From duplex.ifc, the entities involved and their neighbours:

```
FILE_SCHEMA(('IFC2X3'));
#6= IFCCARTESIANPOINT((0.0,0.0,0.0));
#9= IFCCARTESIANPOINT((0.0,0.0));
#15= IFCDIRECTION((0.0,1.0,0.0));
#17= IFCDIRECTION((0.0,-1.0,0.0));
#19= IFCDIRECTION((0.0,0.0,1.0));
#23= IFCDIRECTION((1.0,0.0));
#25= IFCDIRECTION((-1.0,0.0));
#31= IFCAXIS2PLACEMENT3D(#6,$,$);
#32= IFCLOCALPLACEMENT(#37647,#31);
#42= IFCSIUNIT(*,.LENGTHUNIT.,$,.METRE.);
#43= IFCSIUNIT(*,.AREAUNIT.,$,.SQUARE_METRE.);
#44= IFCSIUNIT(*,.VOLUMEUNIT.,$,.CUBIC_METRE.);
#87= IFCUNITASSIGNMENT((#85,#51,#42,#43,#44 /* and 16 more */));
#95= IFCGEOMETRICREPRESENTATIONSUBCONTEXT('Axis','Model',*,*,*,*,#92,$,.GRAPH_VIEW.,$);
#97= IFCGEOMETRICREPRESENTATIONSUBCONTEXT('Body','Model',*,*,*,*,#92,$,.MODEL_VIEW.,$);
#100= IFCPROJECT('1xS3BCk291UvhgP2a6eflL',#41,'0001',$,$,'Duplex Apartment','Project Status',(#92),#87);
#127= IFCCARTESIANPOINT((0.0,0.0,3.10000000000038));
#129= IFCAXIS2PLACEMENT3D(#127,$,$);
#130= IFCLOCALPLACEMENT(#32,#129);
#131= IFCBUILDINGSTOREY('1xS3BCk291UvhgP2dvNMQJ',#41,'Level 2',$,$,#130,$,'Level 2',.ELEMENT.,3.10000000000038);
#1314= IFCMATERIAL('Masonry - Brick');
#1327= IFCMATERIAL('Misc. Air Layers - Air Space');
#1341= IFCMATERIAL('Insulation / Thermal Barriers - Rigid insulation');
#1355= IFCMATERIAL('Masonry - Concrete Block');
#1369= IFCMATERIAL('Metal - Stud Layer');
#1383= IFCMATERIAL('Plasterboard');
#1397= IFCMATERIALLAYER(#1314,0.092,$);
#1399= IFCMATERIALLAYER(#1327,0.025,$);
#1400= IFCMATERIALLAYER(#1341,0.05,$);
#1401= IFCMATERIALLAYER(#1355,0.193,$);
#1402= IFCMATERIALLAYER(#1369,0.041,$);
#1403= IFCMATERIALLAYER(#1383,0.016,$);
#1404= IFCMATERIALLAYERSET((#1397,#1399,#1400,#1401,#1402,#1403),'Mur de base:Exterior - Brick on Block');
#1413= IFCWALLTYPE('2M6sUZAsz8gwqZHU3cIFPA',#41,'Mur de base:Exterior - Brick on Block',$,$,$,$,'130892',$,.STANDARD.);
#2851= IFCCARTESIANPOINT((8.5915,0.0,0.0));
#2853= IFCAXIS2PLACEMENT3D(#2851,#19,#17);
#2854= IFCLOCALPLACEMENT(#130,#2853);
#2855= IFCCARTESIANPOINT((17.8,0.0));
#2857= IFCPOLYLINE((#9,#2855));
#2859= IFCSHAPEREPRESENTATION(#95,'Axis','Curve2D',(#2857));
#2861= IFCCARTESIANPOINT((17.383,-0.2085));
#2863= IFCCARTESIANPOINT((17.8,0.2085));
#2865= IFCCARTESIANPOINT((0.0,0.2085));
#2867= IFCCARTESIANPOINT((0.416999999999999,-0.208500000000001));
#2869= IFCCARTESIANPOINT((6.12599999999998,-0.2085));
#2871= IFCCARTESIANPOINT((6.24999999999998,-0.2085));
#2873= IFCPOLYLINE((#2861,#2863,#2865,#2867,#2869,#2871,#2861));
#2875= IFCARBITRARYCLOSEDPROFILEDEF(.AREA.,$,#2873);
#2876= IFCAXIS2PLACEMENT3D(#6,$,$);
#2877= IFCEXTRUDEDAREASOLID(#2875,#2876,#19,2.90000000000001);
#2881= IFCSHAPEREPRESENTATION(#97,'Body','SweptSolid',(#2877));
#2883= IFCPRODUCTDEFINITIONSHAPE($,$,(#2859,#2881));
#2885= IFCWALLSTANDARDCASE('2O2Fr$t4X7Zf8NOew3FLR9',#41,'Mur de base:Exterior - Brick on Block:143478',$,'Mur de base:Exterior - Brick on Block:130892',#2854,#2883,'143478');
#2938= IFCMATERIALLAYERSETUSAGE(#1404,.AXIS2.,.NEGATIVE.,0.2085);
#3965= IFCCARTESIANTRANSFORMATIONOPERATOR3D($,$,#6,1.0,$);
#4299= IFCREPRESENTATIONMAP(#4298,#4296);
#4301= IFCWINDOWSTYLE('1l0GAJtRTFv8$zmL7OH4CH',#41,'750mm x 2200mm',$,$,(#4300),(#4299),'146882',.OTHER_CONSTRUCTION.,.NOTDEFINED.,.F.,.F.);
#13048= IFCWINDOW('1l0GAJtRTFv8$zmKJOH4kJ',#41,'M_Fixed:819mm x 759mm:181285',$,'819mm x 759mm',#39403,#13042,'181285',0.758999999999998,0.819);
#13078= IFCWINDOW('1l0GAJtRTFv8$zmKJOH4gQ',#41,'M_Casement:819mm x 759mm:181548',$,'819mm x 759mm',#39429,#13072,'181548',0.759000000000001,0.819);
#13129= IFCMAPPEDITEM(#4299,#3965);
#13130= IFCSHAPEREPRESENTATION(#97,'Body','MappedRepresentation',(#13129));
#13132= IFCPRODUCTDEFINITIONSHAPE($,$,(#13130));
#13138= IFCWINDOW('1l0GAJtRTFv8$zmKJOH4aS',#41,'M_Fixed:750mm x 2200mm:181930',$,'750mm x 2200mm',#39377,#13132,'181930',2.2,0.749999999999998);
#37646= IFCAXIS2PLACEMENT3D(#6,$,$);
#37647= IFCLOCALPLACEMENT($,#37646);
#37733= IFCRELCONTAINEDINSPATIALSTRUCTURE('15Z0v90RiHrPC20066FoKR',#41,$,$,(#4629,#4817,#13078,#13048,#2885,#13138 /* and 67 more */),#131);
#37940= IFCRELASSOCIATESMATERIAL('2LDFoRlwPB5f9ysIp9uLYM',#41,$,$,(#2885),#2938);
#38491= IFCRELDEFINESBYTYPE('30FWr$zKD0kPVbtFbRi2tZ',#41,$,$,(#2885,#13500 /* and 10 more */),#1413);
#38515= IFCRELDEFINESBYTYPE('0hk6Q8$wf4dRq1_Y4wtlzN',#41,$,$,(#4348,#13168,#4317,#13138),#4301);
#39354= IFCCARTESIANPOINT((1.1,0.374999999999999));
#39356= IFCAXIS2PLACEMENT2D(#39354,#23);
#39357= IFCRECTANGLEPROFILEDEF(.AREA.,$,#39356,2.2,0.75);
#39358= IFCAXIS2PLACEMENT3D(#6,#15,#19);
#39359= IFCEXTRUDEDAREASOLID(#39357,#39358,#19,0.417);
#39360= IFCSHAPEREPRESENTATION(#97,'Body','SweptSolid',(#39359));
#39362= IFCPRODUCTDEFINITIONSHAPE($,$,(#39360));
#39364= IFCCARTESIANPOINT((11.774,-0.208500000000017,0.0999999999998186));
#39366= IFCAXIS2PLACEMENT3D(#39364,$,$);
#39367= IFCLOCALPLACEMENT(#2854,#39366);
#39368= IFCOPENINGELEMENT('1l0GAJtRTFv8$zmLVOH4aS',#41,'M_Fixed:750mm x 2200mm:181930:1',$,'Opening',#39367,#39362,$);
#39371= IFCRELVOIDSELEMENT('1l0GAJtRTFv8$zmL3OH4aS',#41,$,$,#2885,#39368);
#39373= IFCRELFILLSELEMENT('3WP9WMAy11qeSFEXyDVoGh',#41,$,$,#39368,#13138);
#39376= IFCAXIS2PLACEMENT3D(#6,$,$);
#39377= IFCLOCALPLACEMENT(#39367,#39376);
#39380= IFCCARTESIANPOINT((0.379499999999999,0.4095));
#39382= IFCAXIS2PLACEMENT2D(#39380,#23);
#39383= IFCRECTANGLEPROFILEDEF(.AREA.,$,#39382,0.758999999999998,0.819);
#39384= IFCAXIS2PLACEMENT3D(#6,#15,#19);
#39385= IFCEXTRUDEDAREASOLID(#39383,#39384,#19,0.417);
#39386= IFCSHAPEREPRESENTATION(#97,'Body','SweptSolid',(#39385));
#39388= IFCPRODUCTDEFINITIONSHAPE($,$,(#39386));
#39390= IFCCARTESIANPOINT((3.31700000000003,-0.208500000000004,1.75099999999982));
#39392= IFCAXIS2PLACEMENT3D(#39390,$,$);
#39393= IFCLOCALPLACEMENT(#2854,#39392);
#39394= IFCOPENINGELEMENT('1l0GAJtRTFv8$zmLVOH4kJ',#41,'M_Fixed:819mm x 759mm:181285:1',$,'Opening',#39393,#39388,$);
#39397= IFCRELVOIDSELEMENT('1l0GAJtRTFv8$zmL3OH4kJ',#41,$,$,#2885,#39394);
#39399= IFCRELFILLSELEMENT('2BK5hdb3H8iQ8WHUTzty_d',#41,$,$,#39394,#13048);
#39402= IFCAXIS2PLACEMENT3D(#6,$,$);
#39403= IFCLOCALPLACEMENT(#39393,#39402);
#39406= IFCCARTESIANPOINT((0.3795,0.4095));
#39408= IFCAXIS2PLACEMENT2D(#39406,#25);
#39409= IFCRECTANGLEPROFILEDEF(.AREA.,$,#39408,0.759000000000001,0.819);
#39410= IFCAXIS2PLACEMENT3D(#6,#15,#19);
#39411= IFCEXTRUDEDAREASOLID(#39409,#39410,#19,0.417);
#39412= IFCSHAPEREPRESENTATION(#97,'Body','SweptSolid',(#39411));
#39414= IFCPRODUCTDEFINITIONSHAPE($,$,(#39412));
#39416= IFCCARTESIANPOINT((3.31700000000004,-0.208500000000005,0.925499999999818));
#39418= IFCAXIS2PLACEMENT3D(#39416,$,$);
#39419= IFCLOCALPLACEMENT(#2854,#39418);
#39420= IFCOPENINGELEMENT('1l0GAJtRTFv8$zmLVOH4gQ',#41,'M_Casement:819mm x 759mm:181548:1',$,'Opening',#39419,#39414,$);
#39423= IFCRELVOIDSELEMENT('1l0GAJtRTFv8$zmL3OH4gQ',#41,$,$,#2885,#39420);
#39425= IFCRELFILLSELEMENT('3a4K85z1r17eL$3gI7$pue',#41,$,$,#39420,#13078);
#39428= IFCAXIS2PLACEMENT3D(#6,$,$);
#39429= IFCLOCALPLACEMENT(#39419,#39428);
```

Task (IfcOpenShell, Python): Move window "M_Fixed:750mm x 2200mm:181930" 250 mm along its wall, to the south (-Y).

```python
import ifcopenshell
import ifcopenshell.api.geometry
import ifcopenshell.util.placement

model = ifcopenshell.open("duplex.ifc")

window = model.by_guid("1l0GAJtRTFv8$zmKJOH4aS")
opening = window.FillsVoids[0].RelatingOpeningElement
wall = opening.VoidsElements[0].RelatingBuildingElement

wall_matrix = ifcopenshell.util.placement.get_local_placement(wall.ObjectPlacement)
shift = wall_matrix[:3, 0] * 0.25
before = ifcopenshell.util.placement.get_local_placement(window.ObjectPlacement)[:3, 3].copy()

# The window is placed relative to its opening, so it follows when the opening moves.
matrix = ifcopenshell.util.placement.get_local_placement(opening.ObjectPlacement)
matrix[:3, 3] += shift
ifcopenshell.api.geometry.edit_object_placement(
    model, product=opening, matrix=matrix, is_si=False, should_transform_children=True
)

after = ifcopenshell.util.placement.get_local_placement(window.ObjectPlacement)[:3, 3]
print("window moved by", (after - before).round(3) + 0.0)

model.write("duplex_edited.ifc")
```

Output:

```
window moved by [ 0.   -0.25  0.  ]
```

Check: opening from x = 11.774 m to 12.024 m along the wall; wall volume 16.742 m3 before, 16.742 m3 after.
